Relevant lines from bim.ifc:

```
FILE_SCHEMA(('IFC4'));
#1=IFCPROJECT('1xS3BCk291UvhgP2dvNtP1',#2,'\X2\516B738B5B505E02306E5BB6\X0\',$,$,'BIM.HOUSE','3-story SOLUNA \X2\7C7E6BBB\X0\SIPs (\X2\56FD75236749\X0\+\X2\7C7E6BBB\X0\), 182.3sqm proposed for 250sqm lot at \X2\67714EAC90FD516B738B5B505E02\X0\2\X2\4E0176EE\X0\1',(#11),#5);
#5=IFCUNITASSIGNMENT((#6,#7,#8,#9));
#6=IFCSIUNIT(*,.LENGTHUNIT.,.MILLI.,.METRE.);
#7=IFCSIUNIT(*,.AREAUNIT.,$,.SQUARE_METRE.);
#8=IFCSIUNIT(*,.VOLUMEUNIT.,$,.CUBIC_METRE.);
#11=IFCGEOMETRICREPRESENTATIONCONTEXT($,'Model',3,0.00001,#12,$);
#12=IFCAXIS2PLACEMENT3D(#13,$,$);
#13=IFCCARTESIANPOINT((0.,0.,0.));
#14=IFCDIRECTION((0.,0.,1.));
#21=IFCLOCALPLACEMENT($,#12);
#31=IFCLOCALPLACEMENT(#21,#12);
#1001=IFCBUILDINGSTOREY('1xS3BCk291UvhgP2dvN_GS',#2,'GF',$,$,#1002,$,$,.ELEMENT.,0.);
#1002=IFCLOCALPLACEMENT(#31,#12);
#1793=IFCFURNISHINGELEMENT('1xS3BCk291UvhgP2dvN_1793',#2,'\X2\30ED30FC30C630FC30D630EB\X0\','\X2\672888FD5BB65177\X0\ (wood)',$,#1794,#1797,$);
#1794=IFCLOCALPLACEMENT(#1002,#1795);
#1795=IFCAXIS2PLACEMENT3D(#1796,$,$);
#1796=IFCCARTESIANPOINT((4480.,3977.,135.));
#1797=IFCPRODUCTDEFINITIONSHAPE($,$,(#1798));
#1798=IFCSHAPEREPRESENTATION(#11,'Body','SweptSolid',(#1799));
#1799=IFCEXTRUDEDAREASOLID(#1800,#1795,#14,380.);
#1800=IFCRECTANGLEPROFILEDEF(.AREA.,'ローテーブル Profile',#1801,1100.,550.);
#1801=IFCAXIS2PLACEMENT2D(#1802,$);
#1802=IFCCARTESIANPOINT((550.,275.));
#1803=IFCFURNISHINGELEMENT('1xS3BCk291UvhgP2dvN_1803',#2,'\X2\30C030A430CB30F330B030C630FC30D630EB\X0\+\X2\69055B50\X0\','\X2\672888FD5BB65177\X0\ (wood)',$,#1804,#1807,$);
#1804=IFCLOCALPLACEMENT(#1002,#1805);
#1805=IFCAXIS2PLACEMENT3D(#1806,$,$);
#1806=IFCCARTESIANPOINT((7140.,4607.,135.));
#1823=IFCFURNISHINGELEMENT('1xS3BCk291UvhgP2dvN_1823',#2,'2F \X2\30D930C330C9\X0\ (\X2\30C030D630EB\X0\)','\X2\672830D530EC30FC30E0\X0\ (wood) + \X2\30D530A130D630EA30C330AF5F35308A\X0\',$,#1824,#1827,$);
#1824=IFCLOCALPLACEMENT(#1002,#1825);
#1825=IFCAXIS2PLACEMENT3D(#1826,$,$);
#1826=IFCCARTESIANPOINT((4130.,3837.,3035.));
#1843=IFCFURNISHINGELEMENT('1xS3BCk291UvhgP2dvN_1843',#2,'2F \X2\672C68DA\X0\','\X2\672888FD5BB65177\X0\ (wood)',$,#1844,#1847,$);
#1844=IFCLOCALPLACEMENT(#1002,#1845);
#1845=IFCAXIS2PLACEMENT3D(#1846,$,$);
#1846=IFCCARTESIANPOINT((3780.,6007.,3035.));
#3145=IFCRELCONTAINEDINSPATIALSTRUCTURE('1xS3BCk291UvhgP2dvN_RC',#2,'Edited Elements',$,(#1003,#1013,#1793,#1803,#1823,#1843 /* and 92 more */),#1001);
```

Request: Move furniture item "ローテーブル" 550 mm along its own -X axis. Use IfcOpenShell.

```python
import ifcopenshell
import ifcopenshell.api.geometry
import ifcopenshell.util.placement
import ifcopenshell.util.unit

model = ifcopenshell.open("bim.ifc")
unit_scale = ifcopenshell.util.unit.calculate_unit_scale(model)

item = model.by_guid("1xS3BCk291UvhgP2dvN_1793")
matrix = ifcopenshell.util.placement.get_local_placement(item.ObjectPlacement)
matrix[:3, 3] -= matrix[:3, 0] * 0.55 / unit_scale
ifcopenshell.api.geometry.edit_object_placement(model, product=item, matrix=matrix, is_si=False)

print(ifcopenshell.util.placement.get_local_placement(item.ObjectPlacement).round(3) + 0.0)

model.write("bim_rev.ifc")
```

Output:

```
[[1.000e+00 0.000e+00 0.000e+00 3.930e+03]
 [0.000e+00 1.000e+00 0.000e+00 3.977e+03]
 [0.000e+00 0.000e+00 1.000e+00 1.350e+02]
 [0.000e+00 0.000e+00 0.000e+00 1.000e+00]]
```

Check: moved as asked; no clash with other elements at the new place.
